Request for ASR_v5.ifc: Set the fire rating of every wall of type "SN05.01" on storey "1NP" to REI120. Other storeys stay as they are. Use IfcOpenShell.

First a look at what the model holds.

```python
import ifcopenshell
import ifcopenshell.util.element

model = ifcopenshell.open("ASR_v5.ifc")
print(model.schema)
storey = next(s for s in model.by_type("IfcBuildingStorey") if s.Name == "1NP")
walls = [e for e in ifcopenshell.util.element.get_decomposition(storey) if e.is_a("IfcWall")]
seen = {}
for e in walls:
    element_type = ifcopenshell.util.element.get_type(e)
    key = (element_type.Name if element_type != e and element_type else None, ifcopenshell.util.element.get_pset(e, "Pset_WallCommon", "FireRating"))
    seen[key] = seen.get(key, 0) + 1
for (name, value), count in sorted(seen.items(), key=str):
    print(count, "x", name, "|", value)
```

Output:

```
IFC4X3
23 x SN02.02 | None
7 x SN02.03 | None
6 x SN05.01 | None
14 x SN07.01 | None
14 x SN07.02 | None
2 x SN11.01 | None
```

```python
import ifcopenshell
import ifcopenshell.api.pset
import ifcopenshell.util.element

model = ifcopenshell.open("ASR_v5.ifc")

storey = next(s for s in model.by_type("IfcBuildingStorey") if s.Name == "1NP")
walls = [e for e in ifcopenshell.util.element.get_decomposition(storey) if e.is_a("IfcWall")]

count = 0
for e in walls:
    element_type = ifcopenshell.util.element.get_type(e)
    if element_type in (None, e) or element_type.Name != "SN05.01":
        continue
    # add_pset returns the element's existing set when there is one.
    pset = ifcopenshell.api.pset.add_pset(model, product=e, name="Pset_WallCommon")
    ifcopenshell.api.pset.edit_pset(model, pset=pset, properties={"FireRating": "REI120"})
    count += 1

print(count, "walls updated")

model.write("ASR_v5-out.ifc")
```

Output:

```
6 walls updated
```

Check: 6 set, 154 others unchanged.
